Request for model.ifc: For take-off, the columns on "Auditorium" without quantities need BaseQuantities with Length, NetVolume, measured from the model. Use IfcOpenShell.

First a look at what the model holds.

```python
import ifcopenshell
import ifcopenshell.util.element
import ifcopenshell.util.unit

model = ifcopenshell.open("model.ifc")
print(model.schema)
for unit_type in ("LENGTHUNIT", "AREAUNIT", "VOLUMEUNIT"):
    print(unit_type, ifcopenshell.util.unit.calculate_unit_scale(model, unit_type))
storey = next(s for s in model.by_type("IfcBuildingStorey") if s.Name == "Auditorium")
columns = [e for e in ifcopenshell.util.element.get_decomposition(storey) if e.is_a("IfcColumn")]
for e in sorted(columns, key=lambda e: e.id()):
    print(e.id(), e.is_a(), e.Name, list(ifcopenshell.util.element.get_psets(e, qtos_only=True)), sep=" | ")
```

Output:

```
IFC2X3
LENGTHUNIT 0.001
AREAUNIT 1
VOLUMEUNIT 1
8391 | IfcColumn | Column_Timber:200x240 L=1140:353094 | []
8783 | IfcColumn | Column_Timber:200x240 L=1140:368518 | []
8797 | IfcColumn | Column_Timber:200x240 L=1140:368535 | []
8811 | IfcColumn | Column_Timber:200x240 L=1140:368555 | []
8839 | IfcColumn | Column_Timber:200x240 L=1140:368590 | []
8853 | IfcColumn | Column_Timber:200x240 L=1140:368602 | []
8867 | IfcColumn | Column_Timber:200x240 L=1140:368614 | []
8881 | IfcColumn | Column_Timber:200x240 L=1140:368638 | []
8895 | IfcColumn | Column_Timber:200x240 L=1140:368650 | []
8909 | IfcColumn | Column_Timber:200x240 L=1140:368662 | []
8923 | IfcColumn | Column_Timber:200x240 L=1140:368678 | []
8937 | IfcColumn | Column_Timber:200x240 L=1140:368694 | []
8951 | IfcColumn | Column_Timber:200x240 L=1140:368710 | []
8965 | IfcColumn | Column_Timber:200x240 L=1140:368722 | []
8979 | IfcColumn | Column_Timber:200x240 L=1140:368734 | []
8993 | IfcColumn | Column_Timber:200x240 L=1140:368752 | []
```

```python
import ifcopenshell
import ifcopenshell.api.pset
import ifcopenshell.geom
import ifcopenshell.util.element
import ifcopenshell.util.shape
import ifcopenshell.util.unit

model = ifcopenshell.open("model.ifc")
unit_scale = ifcopenshell.util.unit.calculate_unit_scale(model)
volume_scale = ifcopenshell.util.unit.calculate_unit_scale(model, "VOLUMEUNIT")
settings = ifcopenshell.geom.settings()

storey = next(s for s in model.by_type("IfcBuildingStorey") if s.Name == "Auditorium")
columns = [e for e in ifcopenshell.util.element.get_decomposition(storey) if e.is_a("IfcColumn")]

for e in sorted(columns, key=lambda e: e.id()):
    if ifcopenshell.util.element.get_psets(e, qtos_only=True, should_inherit=False):
        continue
    # Geometry comes back in metres, in the element's own axes.
    shape = ifcopenshell.geom.create_shape(settings, e)
    values = {
        "Length": ifcopenshell.util.shape.get_z(shape.geometry) / unit_scale,
        "NetVolume": ifcopenshell.util.shape.get_volume(shape.geometry) / volume_scale,
    }
    qto = ifcopenshell.api.pset.add_qto(model, product=e, name="BaseQuantities")
    ifcopenshell.api.pset.edit_qto(model, qto=qto, properties=values)
    print(e.id(), {k: round(v, 3) for k, v in values.items()})

model.write("model_updated.ifc")
```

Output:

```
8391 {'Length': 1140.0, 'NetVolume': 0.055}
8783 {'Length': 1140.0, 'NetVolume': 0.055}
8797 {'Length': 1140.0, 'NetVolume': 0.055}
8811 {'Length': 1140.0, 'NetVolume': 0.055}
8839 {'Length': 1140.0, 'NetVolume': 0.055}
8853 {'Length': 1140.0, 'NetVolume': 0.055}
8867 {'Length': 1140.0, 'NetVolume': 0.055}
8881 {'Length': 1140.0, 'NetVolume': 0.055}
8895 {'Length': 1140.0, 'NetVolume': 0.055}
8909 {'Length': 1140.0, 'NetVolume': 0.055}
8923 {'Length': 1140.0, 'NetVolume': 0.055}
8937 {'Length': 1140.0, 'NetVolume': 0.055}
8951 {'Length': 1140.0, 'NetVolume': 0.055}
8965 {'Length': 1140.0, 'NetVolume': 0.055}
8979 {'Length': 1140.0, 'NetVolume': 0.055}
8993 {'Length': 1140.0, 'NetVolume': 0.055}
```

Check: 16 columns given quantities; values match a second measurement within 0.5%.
